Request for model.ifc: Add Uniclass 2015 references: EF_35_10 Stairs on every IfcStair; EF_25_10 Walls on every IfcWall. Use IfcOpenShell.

First a look at what the model holds.

```python
import ifcopenshell

model = ifcopenshell.open("model.ifc")
print(model.schema)
print("classifications:", [c.Name for c in model.by_type("IfcClassification")])
for ifc_class in ("IfcDoor", "IfcRoof", "IfcStair", "IfcWall", "IfcWindow"):
    print(ifc_class, len(model.by_type(ifc_class)))
```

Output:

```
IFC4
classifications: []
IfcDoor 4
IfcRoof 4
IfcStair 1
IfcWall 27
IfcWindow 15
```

```python
import ifcopenshell
import ifcopenshell.api.classification

model = ifcopenshell.open("model.ifc")

system = ifcopenshell.api.classification.add_classification(model, classification="Uniclass 2015")

codes = {
    "IfcStair": ("EF_35_10", "Stairs"),
    "IfcWall": ("EF_25_10", "Walls"),
}
for ifc_class, (code, name) in codes.items():
    products = model.by_type(ifc_class)
    ifcopenshell.api.classification.add_reference(
        model, products=products, classification=system, identification=code, name=name
    )
    print(code, len(products))

model.write("model_updated.ifc")
```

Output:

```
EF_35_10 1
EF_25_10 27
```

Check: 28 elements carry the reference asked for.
